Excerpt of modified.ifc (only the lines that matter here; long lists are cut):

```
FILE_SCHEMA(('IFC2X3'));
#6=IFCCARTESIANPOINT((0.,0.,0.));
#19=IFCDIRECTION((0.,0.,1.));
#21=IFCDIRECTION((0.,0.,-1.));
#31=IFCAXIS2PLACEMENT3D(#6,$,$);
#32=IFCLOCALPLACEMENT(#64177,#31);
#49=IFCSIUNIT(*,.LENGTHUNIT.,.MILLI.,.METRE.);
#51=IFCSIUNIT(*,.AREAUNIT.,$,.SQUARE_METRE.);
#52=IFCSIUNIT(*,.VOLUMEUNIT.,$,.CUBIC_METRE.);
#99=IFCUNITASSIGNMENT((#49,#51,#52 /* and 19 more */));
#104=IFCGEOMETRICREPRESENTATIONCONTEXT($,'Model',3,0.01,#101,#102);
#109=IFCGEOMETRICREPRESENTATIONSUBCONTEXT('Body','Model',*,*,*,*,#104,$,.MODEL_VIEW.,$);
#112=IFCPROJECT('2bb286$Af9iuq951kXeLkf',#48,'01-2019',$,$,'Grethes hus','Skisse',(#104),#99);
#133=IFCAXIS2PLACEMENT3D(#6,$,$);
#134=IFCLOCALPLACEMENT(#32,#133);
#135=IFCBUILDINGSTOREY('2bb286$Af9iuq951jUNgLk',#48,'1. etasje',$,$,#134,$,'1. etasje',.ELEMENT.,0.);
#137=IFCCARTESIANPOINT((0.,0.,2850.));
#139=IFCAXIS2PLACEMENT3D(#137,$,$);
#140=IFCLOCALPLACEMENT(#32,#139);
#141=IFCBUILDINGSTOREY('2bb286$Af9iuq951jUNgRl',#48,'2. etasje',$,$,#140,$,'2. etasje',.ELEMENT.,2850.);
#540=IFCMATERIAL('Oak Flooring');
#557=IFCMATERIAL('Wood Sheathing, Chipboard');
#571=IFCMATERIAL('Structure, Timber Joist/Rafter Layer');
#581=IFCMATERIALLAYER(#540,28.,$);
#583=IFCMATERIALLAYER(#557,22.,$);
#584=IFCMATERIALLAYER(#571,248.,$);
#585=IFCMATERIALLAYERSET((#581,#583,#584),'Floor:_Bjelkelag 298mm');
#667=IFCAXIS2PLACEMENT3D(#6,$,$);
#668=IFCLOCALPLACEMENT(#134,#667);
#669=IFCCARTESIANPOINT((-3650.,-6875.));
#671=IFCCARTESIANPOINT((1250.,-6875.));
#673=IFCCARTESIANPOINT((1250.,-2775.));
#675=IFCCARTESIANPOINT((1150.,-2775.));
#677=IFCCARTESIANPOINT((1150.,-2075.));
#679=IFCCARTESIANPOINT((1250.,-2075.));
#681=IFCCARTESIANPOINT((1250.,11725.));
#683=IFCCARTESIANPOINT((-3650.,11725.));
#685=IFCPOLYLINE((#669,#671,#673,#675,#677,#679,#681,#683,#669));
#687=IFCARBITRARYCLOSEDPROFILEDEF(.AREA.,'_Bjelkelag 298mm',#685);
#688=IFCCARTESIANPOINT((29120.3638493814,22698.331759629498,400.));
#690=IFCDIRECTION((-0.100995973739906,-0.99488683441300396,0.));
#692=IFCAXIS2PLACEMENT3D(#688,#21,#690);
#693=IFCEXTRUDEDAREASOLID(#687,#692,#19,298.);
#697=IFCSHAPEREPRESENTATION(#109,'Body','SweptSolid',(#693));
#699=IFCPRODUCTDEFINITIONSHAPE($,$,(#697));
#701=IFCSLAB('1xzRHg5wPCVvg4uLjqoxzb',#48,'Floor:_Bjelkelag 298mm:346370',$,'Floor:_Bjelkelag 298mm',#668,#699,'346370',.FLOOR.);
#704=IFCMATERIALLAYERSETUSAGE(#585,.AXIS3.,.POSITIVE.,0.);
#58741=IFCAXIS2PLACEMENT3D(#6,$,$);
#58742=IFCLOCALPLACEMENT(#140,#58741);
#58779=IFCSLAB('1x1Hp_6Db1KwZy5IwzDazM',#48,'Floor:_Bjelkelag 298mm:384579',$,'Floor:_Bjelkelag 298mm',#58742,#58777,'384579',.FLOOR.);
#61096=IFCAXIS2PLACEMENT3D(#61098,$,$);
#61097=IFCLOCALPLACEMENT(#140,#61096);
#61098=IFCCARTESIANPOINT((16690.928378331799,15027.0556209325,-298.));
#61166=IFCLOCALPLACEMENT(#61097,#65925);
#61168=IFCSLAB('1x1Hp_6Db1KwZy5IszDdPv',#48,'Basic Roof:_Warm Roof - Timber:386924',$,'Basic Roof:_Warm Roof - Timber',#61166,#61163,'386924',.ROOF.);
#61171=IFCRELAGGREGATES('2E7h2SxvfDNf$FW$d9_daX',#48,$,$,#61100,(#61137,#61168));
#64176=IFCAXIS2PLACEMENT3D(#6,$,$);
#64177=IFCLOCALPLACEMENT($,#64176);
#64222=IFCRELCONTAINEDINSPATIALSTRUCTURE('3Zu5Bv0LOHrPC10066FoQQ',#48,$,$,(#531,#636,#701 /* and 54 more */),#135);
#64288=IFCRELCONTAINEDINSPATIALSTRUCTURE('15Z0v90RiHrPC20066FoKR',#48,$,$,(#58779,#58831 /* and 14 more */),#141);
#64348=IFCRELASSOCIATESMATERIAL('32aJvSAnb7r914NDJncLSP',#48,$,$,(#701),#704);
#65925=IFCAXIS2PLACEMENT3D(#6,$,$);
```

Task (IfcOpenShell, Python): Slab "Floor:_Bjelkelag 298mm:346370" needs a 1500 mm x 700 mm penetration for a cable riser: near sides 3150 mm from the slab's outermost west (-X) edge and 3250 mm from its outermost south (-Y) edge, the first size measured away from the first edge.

```python
import numpy as np
import ifcopenshell
import ifcopenshell.api.feature
import ifcopenshell.api.geometry
import ifcopenshell.api.root
import ifcopenshell.geom
import ifcopenshell.util.placement
import ifcopenshell.util.representation
import ifcopenshell.util.shape
import ifcopenshell.util.unit

model = ifcopenshell.open("modified.ifc")
unit_scale = ifcopenshell.util.unit.calculate_unit_scale(model)
settings = ifcopenshell.geom.settings()


def volume(element):
    """Net volume in cubic metres, openings subtracted."""
    shape = ifcopenshell.geom.create_shape(settings, element)
    return ifcopenshell.util.shape.get_volume(shape.geometry)


slab = model.by_guid("1xzRHg5wPCVvg4uLjqoxzb")
before = volume(slab)

# Extent in the slab's own axes, in metres. The edges named are its -X and -Y sides.
slab_shape = ifcopenshell.geom.create_shape(settings, slab)
vertices = ifcopenshell.util.shape.get_vertices(slab_shape.geometry)
x_min, y_min, bottom = vertices.min(axis=0)
top = vertices[:, 2].max()

opening = ifcopenshell.api.root.create_entity(model, ifc_class="IfcOpeningElement", name="Cable riser opening")
context = ifcopenshell.util.representation.get_context(model, "Model", "Body", "MODEL_VIEW")
width, depth = 1.5, 0.7
outline = [(0.0, 0.0), (width, 0.0), (width, depth), (0.0, depth), (0.0, 0.0)]
# Overshoot both faces by 50 mm so the cut is clean.
shape = ifcopenshell.api.geometry.add_slab_representation(
    model, context=context, depth=top - bottom + 0.1, polyline=outline
)
ifcopenshell.api.geometry.assign_representation(model, product=opening, representation=shape)

matrix = ifcopenshell.util.placement.get_local_placement(slab.ObjectPlacement)
matrix[:, 3] = matrix @ np.append(np.array([x_min + 3.15, y_min + 3.25, bottom - 0.05]) / unit_scale, 1.0)
ifcopenshell.api.geometry.edit_object_placement(model, product=opening, matrix=matrix, is_si=False)
ifcopenshell.api.feature.add_feature(model, feature=opening, element=slab)

after = volume(slab)

print(f"slab volume {before:.3f} -> {after:.3f} m3")

model.write("modified_updated.ifc")
```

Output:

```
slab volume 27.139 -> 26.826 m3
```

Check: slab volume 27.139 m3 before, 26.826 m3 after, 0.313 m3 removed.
